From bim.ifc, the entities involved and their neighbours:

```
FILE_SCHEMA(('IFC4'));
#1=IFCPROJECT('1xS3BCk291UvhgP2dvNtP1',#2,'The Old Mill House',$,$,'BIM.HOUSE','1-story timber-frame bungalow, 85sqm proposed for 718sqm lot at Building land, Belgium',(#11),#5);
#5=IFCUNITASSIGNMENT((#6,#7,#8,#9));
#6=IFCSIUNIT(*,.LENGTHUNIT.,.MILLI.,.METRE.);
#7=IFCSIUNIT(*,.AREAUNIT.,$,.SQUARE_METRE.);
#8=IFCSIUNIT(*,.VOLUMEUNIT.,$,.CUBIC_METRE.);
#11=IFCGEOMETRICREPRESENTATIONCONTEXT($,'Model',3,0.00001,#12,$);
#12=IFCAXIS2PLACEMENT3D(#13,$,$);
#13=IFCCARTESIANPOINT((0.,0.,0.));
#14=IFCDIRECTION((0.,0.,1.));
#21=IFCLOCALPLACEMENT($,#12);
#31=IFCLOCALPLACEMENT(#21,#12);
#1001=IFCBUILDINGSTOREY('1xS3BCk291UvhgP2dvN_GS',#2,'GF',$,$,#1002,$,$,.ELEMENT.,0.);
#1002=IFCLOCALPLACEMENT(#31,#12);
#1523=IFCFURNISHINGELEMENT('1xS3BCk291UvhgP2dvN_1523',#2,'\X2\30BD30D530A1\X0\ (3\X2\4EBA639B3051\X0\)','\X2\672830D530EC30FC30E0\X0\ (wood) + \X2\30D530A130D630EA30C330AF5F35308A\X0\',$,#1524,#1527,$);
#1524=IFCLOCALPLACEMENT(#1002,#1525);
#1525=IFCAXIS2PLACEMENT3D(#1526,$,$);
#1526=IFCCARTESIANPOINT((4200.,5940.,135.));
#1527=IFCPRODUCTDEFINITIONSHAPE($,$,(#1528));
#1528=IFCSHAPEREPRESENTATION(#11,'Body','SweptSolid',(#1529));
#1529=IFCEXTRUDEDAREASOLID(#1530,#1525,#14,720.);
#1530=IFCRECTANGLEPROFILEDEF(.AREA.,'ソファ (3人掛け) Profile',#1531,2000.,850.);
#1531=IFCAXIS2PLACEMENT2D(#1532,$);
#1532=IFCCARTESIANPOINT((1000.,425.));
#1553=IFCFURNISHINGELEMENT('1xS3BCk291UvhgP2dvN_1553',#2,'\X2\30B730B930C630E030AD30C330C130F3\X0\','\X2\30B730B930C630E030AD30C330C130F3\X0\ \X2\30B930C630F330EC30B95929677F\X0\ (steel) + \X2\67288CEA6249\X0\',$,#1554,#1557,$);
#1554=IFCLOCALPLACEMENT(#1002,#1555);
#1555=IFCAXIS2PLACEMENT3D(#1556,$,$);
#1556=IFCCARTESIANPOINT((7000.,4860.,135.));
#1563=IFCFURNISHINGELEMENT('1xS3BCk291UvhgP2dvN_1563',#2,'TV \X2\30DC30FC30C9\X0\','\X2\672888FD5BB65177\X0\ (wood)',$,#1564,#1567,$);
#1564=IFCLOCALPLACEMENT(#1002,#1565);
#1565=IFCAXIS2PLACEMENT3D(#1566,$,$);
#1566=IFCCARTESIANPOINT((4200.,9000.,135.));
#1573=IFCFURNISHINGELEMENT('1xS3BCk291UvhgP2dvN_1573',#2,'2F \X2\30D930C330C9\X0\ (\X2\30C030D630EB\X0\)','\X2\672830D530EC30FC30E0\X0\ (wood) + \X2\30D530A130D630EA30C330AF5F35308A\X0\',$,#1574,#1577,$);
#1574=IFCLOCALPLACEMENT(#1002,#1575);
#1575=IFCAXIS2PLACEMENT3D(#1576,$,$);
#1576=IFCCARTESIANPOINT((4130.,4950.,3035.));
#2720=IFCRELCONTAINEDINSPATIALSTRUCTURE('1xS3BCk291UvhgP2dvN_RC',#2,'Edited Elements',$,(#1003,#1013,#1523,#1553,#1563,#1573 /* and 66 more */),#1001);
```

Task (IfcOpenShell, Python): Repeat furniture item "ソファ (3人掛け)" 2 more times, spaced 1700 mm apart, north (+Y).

```python
import numpy as np
import ifcopenshell
import ifcopenshell.api.geometry
import ifcopenshell.api.root
import ifcopenshell.util.element
import ifcopenshell.util.placement
import ifcopenshell.util.unit

model = ifcopenshell.open("bim.ifc")
unit_scale = ifcopenshell.util.unit.calculate_unit_scale(model)


def reuse_history(source, copy):
    """copy_class also copies each property set's owner history, people and application; keep the originals."""
    for rel in copy.IsDefinedBy:
        if rel.is_a("IfcRelDefinesByProperties") and (history := rel.RelatingPropertyDefinition.OwnerHistory):
            rel.RelatingPropertyDefinition.OwnerHistory = source.OwnerHistory
            ifcopenshell.util.element.remove_deep2(model, history)


source = model.by_guid("1xS3BCk291UvhgP2dvN_1523")
base = ifcopenshell.util.placement.get_local_placement(source.ObjectPlacement)
step = np.array([0.0, 1.0, 0.0]) * 1.7 / unit_scale

for i in range(1, 3):
    copy = ifcopenshell.api.root.copy_class(model, product=source)
    copy.Representation = ifcopenshell.util.element.copy_deep(
        model, source.Representation, exclude=["IfcGeometricRepresentationContext", "IfcRepresentationMap"]
    )
    reuse_history(source, copy)
    matrix = base.copy()
    matrix[:3, 3] += i * step
    print("added at", matrix[:3, 3].round(3) + 0.0)
    ifcopenshell.api.geometry.edit_object_placement(model, product=copy, matrix=matrix, is_si=False)

model.write("bim_rev.ifc")
```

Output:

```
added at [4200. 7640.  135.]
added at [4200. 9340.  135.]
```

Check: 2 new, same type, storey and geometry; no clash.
